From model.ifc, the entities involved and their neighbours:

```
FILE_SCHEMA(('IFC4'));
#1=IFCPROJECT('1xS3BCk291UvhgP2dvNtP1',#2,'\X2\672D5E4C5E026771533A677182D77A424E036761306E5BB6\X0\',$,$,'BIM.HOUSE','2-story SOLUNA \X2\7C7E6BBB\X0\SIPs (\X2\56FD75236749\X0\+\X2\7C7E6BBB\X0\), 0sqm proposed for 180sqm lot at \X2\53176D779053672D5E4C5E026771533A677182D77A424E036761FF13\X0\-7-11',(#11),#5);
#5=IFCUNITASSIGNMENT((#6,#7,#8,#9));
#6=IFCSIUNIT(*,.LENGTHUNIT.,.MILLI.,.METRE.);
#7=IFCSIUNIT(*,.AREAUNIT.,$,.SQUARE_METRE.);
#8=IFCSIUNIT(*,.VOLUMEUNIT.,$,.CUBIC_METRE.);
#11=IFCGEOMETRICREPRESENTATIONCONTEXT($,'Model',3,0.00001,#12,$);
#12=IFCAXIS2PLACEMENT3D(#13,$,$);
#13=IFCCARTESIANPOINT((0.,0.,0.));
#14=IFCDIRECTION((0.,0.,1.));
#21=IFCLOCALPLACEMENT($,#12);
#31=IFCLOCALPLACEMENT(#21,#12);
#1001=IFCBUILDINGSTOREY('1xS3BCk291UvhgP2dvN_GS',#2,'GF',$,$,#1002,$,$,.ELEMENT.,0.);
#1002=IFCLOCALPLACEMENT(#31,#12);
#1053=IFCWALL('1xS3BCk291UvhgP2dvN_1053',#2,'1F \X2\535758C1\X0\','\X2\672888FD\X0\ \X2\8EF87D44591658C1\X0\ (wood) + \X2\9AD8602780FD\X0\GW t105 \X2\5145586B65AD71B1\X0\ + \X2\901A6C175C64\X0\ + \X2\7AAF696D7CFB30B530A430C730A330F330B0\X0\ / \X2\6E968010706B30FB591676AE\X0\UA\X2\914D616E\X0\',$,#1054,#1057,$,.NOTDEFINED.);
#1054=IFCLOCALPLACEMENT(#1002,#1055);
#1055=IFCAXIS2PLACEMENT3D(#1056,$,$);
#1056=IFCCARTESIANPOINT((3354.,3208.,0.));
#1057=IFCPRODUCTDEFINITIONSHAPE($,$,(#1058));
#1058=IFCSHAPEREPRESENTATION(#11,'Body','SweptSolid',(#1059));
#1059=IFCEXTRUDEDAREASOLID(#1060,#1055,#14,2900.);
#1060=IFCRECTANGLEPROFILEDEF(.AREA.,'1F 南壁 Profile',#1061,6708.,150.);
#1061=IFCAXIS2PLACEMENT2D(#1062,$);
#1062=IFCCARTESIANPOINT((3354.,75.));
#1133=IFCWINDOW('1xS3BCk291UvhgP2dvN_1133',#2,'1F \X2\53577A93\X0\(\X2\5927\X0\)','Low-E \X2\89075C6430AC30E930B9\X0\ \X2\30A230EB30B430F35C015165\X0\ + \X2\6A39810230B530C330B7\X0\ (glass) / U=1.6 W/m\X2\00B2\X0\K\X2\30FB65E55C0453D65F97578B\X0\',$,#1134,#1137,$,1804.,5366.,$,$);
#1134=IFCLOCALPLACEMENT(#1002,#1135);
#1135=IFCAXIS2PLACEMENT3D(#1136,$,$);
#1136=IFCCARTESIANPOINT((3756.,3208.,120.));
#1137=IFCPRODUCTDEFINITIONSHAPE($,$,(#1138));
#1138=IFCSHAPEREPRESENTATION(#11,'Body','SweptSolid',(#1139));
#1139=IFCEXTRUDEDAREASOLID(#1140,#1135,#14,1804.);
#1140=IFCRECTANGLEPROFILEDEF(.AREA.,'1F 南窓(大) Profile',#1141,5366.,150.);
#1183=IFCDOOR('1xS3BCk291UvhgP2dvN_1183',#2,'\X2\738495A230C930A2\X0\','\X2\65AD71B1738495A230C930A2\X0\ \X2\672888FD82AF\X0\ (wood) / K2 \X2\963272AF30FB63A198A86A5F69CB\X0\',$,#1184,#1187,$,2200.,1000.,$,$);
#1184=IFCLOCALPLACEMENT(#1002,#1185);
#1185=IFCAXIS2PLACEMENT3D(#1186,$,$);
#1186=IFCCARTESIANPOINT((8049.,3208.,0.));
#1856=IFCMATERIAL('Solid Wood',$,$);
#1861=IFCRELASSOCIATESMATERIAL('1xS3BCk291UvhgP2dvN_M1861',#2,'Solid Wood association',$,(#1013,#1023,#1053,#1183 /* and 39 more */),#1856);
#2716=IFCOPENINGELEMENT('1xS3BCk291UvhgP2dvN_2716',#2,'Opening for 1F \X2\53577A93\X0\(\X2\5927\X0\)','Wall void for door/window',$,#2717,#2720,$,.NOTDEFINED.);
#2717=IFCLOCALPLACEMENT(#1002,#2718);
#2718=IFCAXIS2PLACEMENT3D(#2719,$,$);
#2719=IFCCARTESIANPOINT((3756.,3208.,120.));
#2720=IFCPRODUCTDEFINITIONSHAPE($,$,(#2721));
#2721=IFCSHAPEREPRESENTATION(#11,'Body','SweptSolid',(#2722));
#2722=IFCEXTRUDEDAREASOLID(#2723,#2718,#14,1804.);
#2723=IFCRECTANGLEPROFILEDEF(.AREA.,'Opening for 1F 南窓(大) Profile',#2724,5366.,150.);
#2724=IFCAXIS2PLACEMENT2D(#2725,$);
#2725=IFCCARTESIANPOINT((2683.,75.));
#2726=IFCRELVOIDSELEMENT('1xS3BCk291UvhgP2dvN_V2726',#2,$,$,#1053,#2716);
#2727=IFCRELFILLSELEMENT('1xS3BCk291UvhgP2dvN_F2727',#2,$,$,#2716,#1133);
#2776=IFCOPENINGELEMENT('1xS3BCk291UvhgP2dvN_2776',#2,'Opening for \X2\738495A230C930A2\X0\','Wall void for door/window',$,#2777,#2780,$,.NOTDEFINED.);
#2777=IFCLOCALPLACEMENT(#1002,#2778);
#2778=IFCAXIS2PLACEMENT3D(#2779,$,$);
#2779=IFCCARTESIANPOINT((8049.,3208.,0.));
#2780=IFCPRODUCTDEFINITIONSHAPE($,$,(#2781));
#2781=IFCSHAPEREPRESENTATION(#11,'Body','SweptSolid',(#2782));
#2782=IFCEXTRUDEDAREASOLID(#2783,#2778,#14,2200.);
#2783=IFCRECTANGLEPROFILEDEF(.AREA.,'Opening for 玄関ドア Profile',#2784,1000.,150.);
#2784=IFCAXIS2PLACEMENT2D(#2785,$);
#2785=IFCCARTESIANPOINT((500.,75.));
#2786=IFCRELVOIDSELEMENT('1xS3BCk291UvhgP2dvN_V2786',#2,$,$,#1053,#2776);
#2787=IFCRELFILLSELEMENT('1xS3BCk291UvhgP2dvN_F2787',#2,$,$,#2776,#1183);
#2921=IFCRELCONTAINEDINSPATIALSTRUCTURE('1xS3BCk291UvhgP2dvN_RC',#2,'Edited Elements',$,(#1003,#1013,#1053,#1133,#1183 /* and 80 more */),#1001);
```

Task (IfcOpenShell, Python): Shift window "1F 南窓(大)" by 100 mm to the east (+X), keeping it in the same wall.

```python
import ifcopenshell
import ifcopenshell.api.geometry
import ifcopenshell.util.placement

model = ifcopenshell.open("model.ifc")

window = model.by_guid("1xS3BCk291UvhgP2dvN_1133")
opening = window.FillsVoids[0].RelatingOpeningElement
wall = opening.VoidsElements[0].RelatingBuildingElement

wall_matrix = ifcopenshell.util.placement.get_local_placement(wall.ObjectPlacement)
shift = wall_matrix[:3, 0] * 100.0
before = ifcopenshell.util.placement.get_local_placement(window.ObjectPlacement)[:3, 3].copy()

# The window is not placed relative to its opening, so move both.
for product in (opening, window):
    matrix = ifcopenshell.util.placement.get_local_placement(product.ObjectPlacement)
    matrix[:3, 3] += shift
    ifcopenshell.api.geometry.edit_object_placement(model, product=product, matrix=matrix, is_si=False)

after = ifcopenshell.util.placement.get_local_placement(window.ObjectPlacement)[:3, 3]
print("window moved by", (after - before).round(3) + 0.0)

model.write("model_rev.ifc")
```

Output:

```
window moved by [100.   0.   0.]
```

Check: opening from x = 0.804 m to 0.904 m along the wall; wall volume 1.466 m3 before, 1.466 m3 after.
